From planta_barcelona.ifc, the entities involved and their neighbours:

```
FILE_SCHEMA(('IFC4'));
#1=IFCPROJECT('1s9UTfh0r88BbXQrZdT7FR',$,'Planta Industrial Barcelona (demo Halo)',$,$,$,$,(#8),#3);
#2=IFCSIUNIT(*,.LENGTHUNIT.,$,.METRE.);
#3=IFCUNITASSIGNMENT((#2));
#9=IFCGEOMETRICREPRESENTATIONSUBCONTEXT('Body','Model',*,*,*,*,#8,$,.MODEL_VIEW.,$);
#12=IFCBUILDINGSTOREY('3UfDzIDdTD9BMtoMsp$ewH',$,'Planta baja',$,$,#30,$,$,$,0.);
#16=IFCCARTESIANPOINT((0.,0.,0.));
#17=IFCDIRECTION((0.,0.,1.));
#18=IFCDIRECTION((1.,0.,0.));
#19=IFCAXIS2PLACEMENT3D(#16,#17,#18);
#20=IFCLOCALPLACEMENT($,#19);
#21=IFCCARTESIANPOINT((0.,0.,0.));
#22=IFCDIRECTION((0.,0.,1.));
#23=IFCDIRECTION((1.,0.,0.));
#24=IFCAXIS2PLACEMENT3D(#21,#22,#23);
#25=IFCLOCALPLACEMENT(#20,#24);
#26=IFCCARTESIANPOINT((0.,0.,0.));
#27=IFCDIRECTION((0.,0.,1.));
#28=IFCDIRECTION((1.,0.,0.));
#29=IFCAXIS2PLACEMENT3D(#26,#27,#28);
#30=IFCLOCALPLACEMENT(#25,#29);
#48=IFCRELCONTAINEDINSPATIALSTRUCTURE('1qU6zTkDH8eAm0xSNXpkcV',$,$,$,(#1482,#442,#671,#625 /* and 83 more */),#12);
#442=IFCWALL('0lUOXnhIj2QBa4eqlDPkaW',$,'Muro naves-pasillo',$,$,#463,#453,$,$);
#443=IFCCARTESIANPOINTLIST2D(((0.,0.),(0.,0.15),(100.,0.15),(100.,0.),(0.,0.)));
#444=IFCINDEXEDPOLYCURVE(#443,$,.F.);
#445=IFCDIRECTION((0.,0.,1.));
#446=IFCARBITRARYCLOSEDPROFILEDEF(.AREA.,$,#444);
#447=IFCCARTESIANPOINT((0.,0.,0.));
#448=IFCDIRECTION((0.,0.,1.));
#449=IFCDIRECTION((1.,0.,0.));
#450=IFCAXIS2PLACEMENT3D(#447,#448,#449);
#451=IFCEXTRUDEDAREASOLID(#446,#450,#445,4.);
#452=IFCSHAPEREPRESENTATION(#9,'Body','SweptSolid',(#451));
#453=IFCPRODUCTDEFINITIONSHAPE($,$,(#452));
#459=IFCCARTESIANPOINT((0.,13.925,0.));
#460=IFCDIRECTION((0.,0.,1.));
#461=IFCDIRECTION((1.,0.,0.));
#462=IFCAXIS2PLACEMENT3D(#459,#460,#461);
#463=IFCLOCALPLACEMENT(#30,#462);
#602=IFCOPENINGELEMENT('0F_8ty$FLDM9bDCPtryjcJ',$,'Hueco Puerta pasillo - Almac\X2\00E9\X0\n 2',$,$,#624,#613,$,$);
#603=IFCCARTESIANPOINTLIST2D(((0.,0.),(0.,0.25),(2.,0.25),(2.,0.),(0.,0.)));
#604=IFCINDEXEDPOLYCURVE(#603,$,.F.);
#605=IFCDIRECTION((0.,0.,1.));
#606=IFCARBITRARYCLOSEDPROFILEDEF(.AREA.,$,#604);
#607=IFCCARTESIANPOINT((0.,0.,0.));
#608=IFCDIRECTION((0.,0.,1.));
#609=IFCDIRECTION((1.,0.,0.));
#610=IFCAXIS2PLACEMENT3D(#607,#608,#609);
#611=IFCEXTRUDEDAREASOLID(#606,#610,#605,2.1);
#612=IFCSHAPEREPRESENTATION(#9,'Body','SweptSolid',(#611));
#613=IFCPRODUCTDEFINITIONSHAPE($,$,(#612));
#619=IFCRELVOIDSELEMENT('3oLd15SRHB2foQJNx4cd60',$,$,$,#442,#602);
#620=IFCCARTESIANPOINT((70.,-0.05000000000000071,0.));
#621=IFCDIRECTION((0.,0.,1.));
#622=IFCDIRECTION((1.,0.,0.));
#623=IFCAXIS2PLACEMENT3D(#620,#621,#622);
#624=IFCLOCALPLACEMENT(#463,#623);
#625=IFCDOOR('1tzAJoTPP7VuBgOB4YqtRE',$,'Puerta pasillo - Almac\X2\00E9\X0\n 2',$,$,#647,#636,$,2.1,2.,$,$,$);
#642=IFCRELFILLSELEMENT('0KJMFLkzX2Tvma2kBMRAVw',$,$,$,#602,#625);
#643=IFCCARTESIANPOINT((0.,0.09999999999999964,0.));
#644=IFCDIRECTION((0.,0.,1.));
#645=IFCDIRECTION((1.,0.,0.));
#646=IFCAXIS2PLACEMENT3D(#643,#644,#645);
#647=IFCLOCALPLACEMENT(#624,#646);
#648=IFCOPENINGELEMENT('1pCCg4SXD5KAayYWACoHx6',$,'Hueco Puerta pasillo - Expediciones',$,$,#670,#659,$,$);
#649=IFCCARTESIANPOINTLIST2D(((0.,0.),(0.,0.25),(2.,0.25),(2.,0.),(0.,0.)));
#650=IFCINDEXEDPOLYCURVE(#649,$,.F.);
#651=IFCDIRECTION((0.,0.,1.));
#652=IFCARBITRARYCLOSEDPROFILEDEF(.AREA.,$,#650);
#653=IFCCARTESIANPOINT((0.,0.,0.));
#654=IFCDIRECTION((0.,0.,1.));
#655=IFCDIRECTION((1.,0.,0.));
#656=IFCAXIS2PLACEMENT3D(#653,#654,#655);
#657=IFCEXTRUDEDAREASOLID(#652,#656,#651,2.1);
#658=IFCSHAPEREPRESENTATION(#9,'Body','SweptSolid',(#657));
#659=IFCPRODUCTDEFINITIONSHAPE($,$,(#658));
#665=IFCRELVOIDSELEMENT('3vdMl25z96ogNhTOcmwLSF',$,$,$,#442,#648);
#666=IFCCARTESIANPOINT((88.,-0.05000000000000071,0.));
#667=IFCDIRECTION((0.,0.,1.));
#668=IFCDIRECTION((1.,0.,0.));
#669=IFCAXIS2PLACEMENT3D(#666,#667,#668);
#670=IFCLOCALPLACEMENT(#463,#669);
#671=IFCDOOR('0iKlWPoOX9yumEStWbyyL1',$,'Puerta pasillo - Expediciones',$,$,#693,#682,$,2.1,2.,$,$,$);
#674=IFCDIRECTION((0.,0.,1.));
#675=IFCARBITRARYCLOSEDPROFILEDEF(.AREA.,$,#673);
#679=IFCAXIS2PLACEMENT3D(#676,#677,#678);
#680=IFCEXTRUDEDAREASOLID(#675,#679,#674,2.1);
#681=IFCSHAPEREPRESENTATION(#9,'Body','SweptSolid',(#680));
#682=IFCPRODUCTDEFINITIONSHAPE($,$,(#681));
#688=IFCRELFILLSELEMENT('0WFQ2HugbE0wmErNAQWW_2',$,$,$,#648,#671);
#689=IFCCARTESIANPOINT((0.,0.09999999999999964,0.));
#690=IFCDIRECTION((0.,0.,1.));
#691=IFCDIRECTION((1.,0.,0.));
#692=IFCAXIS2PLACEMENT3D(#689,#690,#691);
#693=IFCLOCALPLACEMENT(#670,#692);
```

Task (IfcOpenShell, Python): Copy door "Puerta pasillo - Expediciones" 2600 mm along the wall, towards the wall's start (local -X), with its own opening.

```python
import ifcopenshell
import ifcopenshell.api.feature
import ifcopenshell.api.geometry
import ifcopenshell.api.root
import ifcopenshell.geom
import ifcopenshell.util.element
import ifcopenshell.util.placement
import ifcopenshell.util.shape

model = ifcopenshell.open("planta_barcelona.ifc")
settings = ifcopenshell.geom.settings()


def volume(element):
    """Net volume in cubic metres, openings subtracted."""
    shape = ifcopenshell.geom.create_shape(settings, element)
    return ifcopenshell.util.shape.get_volume(shape.geometry)


door = model.by_guid("0iKlWPoOX9yumEStWbyyL1")
opening = door.FillsVoids[0].RelatingOpeningElement
wall = opening.VoidsElements[0].RelatingBuildingElement
before = volume(wall)
shift = ifcopenshell.util.placement.get_local_placement(wall.ObjectPlacement)[:3, 0] * -2.6

# copy_class copies the void relationship, type, container and properties, but no geometry.
new_opening = ifcopenshell.api.root.copy_class(model, product=opening)
new_opening.Representation = ifcopenshell.util.element.copy_deep(
    model, opening.Representation, exclude=["IfcGeometricRepresentationContext", "IfcRepresentationMap"]
)
new_door = ifcopenshell.api.root.copy_class(model, product=door)
new_door.Representation = ifcopenshell.util.element.copy_deep(
    model, door.Representation, exclude=["IfcGeometricRepresentationContext", "IfcRepresentationMap"]
)
ifcopenshell.api.feature.add_filling(model, opening=new_opening, element=new_door)

for old, new in ((opening, new_opening), (door, new_door)):
    matrix = ifcopenshell.util.placement.get_local_placement(old.ObjectPlacement)
    matrix[:3, 3] += shift
    ifcopenshell.api.geometry.edit_object_placement(model, product=new, matrix=matrix, is_si=False)

after = volume(wall)

print(f"wall volume {before:.3f} -> {after:.3f} m3")

model.write("planta_barcelona_updated.ifc")
```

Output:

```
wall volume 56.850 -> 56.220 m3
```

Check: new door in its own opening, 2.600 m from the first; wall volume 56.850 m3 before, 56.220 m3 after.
